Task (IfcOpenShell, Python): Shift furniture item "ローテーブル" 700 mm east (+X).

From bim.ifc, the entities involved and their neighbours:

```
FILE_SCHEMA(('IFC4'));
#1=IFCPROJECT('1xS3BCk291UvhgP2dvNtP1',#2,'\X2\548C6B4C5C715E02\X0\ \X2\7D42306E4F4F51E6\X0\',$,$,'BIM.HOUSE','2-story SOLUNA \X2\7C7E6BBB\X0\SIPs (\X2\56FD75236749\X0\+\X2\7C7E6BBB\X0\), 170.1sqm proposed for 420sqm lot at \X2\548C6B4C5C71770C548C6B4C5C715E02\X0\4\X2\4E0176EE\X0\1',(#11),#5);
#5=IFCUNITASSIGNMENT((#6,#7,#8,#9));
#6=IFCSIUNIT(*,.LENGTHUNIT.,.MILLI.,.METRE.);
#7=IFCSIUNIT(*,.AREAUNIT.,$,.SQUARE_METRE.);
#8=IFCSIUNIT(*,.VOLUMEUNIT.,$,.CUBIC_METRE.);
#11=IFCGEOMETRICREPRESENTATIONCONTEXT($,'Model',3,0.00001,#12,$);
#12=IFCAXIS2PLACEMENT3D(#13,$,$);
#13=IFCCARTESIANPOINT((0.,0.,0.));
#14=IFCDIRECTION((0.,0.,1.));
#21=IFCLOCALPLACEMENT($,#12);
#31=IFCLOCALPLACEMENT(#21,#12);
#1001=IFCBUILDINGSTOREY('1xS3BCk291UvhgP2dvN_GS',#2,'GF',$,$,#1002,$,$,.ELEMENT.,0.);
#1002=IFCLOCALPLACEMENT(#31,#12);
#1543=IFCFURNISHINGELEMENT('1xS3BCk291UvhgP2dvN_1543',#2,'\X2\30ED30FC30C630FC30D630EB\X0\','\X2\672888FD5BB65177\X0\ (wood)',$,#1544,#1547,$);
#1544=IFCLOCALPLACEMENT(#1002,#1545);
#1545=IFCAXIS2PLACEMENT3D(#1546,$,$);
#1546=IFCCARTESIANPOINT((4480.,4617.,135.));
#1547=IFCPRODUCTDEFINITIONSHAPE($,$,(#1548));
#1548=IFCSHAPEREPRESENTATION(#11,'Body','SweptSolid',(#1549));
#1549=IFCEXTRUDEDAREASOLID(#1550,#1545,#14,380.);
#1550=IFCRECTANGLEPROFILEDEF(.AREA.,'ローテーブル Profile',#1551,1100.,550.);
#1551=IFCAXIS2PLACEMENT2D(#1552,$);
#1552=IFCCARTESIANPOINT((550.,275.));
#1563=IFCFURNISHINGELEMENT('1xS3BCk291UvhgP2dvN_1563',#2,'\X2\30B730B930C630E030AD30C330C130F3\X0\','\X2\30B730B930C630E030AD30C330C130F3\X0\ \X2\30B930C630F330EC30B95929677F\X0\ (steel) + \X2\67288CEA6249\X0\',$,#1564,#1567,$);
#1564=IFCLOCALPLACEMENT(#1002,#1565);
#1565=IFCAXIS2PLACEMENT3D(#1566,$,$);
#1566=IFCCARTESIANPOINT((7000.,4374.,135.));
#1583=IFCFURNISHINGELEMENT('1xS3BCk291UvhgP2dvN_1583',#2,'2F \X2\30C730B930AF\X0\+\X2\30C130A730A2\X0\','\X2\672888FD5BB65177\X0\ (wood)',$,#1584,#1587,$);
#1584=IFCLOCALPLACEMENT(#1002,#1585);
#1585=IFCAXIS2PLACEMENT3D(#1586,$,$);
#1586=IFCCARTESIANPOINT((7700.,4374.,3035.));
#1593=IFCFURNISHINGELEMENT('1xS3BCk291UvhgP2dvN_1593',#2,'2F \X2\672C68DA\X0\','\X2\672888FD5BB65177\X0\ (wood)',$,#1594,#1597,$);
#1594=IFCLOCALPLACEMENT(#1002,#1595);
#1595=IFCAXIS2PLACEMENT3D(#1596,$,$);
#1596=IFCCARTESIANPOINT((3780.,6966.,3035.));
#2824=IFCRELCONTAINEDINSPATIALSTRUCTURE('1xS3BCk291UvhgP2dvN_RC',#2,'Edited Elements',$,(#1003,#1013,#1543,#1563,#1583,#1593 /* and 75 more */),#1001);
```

```python
import ifcopenshell
import ifcopenshell.api.geometry
import ifcopenshell.util.placement
import ifcopenshell.util.unit

model = ifcopenshell.open("bim.ifc")
unit_scale = ifcopenshell.util.unit.calculate_unit_scale(model)

item = model.by_guid("1xS3BCk291UvhgP2dvN_1543")
matrix = ifcopenshell.util.placement.get_local_placement(item.ObjectPlacement)
matrix[0, 3] += 0.7 / unit_scale
ifcopenshell.api.geometry.edit_object_placement(model, product=item, matrix=matrix, is_si=False)

print(ifcopenshell.util.placement.get_local_placement(item.ObjectPlacement).round(3) + 0.0)

model.write("bim_updated.ifc")
```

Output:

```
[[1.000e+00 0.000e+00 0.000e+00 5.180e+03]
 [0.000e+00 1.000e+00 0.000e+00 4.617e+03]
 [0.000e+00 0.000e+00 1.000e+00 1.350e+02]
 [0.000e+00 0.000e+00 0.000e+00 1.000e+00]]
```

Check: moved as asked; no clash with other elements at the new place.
